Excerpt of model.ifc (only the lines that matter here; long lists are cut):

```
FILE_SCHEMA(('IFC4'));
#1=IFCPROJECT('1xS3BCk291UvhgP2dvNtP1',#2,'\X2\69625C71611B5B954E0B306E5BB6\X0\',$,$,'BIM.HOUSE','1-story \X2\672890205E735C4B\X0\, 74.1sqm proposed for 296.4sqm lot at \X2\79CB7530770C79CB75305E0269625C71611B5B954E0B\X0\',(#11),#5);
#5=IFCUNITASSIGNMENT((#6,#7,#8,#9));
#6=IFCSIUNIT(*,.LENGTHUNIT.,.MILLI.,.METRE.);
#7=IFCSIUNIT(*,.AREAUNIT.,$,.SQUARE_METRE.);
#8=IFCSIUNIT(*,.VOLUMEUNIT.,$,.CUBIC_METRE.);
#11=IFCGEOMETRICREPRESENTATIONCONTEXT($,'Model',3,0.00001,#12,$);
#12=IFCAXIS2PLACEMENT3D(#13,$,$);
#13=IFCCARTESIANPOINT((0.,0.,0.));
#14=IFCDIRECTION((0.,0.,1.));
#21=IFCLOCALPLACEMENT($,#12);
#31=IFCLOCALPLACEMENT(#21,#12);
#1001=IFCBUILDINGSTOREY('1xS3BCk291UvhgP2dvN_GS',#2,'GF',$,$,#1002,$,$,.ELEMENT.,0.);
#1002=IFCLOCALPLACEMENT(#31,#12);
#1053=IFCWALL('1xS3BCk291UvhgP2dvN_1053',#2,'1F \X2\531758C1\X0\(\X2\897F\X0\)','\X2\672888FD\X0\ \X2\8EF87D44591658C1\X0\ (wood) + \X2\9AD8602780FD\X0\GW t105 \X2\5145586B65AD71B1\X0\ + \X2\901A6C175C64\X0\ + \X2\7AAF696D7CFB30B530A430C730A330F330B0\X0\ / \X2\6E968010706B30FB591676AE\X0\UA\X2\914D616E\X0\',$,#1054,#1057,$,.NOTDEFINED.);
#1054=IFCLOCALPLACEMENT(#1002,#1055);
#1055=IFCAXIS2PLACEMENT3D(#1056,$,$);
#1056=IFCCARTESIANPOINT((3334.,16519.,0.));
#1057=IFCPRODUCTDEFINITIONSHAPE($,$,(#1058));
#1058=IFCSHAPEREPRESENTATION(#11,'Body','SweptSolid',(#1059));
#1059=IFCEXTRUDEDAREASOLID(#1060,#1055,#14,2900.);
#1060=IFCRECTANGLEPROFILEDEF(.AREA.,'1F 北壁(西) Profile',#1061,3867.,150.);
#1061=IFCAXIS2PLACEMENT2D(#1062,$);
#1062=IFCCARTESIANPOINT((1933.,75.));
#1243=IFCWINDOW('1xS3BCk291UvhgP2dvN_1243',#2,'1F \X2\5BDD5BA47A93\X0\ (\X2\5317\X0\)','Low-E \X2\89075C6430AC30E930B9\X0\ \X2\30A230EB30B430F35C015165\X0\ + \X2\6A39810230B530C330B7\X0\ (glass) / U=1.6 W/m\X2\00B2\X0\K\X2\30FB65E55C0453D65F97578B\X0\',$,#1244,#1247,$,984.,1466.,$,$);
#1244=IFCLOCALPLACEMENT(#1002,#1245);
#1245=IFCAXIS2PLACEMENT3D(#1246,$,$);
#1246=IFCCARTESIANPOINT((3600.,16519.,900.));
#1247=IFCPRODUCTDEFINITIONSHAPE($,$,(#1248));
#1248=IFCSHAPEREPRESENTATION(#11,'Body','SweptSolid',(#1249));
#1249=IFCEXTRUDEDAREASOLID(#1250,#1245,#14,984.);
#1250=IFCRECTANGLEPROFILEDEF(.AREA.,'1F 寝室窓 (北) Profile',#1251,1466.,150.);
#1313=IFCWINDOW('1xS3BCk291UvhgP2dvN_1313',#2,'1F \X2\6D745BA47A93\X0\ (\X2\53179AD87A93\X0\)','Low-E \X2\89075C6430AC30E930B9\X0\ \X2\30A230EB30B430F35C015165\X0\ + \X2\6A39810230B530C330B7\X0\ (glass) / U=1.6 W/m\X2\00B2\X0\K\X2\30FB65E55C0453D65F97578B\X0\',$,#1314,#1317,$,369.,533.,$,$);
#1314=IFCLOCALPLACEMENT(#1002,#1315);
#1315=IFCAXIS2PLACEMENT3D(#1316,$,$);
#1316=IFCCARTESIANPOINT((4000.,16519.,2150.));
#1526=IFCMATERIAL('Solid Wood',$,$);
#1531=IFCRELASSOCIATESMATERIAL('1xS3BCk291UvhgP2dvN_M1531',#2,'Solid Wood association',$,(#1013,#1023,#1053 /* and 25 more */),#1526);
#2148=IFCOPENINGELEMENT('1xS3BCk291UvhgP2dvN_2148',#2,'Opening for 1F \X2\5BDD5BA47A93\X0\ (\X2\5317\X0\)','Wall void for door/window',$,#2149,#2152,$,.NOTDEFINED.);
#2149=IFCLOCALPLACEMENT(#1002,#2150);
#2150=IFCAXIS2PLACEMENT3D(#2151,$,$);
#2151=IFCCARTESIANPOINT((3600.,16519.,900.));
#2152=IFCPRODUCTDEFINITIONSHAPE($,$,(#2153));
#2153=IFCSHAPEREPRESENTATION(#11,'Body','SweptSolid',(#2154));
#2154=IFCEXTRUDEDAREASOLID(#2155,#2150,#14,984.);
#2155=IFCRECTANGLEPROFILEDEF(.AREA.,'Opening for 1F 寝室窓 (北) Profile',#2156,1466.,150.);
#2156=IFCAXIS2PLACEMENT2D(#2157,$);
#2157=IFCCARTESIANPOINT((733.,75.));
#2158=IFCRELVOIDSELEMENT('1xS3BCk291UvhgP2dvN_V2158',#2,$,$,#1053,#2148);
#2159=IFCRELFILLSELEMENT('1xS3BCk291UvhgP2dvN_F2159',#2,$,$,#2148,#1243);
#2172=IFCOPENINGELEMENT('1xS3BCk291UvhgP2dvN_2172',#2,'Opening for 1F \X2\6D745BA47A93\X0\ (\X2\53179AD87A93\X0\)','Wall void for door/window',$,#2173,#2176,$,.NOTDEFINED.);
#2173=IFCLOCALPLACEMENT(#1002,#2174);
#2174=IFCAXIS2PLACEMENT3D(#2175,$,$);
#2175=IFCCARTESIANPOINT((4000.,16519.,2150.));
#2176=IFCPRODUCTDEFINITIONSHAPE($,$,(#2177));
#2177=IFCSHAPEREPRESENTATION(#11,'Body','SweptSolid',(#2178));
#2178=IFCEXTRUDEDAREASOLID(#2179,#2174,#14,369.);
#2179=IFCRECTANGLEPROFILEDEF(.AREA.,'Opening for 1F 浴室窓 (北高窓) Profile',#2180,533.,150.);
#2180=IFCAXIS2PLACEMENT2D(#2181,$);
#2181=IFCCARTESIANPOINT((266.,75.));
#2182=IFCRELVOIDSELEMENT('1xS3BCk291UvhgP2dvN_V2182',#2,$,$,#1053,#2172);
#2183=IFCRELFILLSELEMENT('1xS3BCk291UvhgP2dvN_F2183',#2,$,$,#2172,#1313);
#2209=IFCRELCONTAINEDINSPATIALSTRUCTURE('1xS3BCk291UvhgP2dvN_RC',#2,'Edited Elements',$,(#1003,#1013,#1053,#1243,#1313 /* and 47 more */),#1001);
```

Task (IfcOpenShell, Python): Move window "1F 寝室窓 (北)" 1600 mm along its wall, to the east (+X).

```python
import ifcopenshell
import ifcopenshell.api.geometry
import ifcopenshell.util.placement

model = ifcopenshell.open("model.ifc")

window = model.by_guid("1xS3BCk291UvhgP2dvN_1243")
opening = window.FillsVoids[0].RelatingOpeningElement
wall = opening.VoidsElements[0].RelatingBuildingElement

wall_matrix = ifcopenshell.util.placement.get_local_placement(wall.ObjectPlacement)
shift = wall_matrix[:3, 0] * 1600.0
before = ifcopenshell.util.placement.get_local_placement(window.ObjectPlacement)[:3, 3].copy()

# The window is not placed relative to its opening, so move both.
for product in (opening, window):
    matrix = ifcopenshell.util.placement.get_local_placement(product.ObjectPlacement)
    matrix[:3, 3] += shift
    ifcopenshell.api.geometry.edit_object_placement(model, product=product, matrix=matrix, is_si=False)

after = ifcopenshell.util.placement.get_local_placement(window.ObjectPlacement)[:3, 3]
print("window moved by", (after - before).round(3) + 0.0)

model.write("model_v2.ifc")
```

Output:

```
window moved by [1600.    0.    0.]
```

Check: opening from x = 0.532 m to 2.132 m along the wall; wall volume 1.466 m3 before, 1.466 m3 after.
